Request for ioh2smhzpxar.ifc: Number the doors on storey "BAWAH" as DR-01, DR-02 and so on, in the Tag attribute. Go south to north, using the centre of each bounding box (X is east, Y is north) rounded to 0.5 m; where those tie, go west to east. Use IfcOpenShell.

First a look at what the model holds.

```python
import ifcopenshell
import ifcopenshell.util.element
import ifcopenshell.util.placement

model = ifcopenshell.open("ioh2smhzpxar.ifc")
print(model.schema)
storey = next(s for s in model.by_type("IfcBuildingStorey") if s.Name == "BAWAH")
doors = [e for e in ifcopenshell.util.element.get_decomposition(storey) if e.is_a("IfcDoor")]
for e in sorted(doors, key=lambda e: e.id()):
    origin = ifcopenshell.util.placement.get_local_placement(e.ObjectPlacement)[:3, 3]
    print(e.id(), e.Tag, e.Name, origin.round(2) + 0.0, sep=" | ")
```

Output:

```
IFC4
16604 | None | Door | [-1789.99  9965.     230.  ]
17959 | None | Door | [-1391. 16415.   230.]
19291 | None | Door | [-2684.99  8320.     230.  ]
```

```python
import ifcopenshell
import ifcopenshell.geom
import ifcopenshell.util.element
import ifcopenshell.util.shape

model = ifcopenshell.open("ioh2smhzpxar.ifc")
settings = ifcopenshell.geom.settings()
settings.set("use-world-coords", True)


def centre(element):
    shape = ifcopenshell.geom.create_shape(settings, element)
    return ifcopenshell.util.shape.get_bbox_centroid(shape.geometry)


storey = next(s for s in model.by_type("IfcBuildingStorey") if s.Name == "BAWAH")
doors = [e for e in ifcopenshell.util.element.get_decomposition(storey) if e.is_a("IfcDoor")]

# Insertion points can sit at a corner or the storey origin, so sort by the geometry (in metres).
centres = {e: centre(e) for e in doors}
doors.sort(key=lambda e: (round(centres[e][1] / 0.5), centres[e][0]))

for i, e in enumerate(doors, start=1):
    number = f"DR-{i:02d}"
    e.Tag = number
    print(e.id(), number)

model.write("ioh2smhzpxar_updated.ifc")
```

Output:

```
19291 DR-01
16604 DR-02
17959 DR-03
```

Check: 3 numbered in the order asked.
